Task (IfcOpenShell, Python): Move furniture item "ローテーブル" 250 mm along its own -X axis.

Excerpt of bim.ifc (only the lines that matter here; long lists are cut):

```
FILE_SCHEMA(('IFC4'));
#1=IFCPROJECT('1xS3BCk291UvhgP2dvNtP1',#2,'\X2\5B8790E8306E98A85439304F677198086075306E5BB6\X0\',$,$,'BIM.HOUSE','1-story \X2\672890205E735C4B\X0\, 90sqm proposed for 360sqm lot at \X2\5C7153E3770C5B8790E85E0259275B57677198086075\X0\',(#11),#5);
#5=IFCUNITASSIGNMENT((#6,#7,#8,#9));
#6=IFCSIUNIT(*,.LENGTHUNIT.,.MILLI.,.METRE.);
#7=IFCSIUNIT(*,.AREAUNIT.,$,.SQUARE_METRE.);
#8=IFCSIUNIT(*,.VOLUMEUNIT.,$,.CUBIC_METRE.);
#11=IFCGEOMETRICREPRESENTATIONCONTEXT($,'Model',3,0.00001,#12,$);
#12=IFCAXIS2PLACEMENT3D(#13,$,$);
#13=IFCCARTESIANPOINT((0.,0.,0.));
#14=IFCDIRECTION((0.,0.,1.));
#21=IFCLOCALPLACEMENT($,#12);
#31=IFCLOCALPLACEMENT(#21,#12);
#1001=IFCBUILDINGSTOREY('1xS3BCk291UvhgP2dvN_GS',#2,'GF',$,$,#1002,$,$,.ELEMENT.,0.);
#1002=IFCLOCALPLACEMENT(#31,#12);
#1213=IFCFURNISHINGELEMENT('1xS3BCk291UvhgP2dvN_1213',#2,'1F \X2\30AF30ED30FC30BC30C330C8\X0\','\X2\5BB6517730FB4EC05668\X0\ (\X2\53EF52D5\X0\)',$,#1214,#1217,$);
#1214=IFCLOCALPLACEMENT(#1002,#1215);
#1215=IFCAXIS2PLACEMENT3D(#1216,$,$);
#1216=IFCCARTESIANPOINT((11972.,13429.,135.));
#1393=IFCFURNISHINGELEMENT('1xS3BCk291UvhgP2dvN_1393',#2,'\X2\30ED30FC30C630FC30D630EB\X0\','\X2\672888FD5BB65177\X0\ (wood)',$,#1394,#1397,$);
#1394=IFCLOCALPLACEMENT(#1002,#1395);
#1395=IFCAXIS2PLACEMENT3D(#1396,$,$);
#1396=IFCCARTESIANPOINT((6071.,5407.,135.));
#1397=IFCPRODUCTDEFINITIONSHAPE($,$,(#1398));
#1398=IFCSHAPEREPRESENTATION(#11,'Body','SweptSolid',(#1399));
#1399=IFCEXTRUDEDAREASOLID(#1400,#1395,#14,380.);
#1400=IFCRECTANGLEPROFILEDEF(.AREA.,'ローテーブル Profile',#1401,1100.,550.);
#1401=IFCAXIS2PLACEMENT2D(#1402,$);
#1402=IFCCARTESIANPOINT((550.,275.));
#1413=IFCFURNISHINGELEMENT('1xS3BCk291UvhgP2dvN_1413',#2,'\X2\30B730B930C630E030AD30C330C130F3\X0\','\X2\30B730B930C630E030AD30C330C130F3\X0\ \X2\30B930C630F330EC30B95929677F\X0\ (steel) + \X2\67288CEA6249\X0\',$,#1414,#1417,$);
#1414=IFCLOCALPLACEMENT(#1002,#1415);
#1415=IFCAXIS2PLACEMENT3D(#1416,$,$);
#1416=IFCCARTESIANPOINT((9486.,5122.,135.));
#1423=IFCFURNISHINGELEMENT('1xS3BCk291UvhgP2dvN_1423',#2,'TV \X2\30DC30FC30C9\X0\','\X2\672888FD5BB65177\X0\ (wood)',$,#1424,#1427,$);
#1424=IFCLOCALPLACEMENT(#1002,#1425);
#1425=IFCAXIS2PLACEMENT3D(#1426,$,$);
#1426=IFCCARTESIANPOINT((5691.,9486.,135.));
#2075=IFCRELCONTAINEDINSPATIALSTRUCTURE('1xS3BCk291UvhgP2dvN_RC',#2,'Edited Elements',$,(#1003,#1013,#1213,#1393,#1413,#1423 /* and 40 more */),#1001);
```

```python
import ifcopenshell
import ifcopenshell.api.geometry
import ifcopenshell.util.placement
import ifcopenshell.util.unit

model = ifcopenshell.open("bim.ifc")
unit_scale = ifcopenshell.util.unit.calculate_unit_scale(model)

item = model.by_guid("1xS3BCk291UvhgP2dvN_1393")
matrix = ifcopenshell.util.placement.get_local_placement(item.ObjectPlacement)
matrix[:3, 3] -= matrix[:3, 0] * 0.25 / unit_scale
ifcopenshell.api.geometry.edit_object_placement(model, product=item, matrix=matrix, is_si=False)

print(ifcopenshell.util.placement.get_local_placement(item.ObjectPlacement).round(3) + 0.0)

model.write("bim_updated.ifc")
```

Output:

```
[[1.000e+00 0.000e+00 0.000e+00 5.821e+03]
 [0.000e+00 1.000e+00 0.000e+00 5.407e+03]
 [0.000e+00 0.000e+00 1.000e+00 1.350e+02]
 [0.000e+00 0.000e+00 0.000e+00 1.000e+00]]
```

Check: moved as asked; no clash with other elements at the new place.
